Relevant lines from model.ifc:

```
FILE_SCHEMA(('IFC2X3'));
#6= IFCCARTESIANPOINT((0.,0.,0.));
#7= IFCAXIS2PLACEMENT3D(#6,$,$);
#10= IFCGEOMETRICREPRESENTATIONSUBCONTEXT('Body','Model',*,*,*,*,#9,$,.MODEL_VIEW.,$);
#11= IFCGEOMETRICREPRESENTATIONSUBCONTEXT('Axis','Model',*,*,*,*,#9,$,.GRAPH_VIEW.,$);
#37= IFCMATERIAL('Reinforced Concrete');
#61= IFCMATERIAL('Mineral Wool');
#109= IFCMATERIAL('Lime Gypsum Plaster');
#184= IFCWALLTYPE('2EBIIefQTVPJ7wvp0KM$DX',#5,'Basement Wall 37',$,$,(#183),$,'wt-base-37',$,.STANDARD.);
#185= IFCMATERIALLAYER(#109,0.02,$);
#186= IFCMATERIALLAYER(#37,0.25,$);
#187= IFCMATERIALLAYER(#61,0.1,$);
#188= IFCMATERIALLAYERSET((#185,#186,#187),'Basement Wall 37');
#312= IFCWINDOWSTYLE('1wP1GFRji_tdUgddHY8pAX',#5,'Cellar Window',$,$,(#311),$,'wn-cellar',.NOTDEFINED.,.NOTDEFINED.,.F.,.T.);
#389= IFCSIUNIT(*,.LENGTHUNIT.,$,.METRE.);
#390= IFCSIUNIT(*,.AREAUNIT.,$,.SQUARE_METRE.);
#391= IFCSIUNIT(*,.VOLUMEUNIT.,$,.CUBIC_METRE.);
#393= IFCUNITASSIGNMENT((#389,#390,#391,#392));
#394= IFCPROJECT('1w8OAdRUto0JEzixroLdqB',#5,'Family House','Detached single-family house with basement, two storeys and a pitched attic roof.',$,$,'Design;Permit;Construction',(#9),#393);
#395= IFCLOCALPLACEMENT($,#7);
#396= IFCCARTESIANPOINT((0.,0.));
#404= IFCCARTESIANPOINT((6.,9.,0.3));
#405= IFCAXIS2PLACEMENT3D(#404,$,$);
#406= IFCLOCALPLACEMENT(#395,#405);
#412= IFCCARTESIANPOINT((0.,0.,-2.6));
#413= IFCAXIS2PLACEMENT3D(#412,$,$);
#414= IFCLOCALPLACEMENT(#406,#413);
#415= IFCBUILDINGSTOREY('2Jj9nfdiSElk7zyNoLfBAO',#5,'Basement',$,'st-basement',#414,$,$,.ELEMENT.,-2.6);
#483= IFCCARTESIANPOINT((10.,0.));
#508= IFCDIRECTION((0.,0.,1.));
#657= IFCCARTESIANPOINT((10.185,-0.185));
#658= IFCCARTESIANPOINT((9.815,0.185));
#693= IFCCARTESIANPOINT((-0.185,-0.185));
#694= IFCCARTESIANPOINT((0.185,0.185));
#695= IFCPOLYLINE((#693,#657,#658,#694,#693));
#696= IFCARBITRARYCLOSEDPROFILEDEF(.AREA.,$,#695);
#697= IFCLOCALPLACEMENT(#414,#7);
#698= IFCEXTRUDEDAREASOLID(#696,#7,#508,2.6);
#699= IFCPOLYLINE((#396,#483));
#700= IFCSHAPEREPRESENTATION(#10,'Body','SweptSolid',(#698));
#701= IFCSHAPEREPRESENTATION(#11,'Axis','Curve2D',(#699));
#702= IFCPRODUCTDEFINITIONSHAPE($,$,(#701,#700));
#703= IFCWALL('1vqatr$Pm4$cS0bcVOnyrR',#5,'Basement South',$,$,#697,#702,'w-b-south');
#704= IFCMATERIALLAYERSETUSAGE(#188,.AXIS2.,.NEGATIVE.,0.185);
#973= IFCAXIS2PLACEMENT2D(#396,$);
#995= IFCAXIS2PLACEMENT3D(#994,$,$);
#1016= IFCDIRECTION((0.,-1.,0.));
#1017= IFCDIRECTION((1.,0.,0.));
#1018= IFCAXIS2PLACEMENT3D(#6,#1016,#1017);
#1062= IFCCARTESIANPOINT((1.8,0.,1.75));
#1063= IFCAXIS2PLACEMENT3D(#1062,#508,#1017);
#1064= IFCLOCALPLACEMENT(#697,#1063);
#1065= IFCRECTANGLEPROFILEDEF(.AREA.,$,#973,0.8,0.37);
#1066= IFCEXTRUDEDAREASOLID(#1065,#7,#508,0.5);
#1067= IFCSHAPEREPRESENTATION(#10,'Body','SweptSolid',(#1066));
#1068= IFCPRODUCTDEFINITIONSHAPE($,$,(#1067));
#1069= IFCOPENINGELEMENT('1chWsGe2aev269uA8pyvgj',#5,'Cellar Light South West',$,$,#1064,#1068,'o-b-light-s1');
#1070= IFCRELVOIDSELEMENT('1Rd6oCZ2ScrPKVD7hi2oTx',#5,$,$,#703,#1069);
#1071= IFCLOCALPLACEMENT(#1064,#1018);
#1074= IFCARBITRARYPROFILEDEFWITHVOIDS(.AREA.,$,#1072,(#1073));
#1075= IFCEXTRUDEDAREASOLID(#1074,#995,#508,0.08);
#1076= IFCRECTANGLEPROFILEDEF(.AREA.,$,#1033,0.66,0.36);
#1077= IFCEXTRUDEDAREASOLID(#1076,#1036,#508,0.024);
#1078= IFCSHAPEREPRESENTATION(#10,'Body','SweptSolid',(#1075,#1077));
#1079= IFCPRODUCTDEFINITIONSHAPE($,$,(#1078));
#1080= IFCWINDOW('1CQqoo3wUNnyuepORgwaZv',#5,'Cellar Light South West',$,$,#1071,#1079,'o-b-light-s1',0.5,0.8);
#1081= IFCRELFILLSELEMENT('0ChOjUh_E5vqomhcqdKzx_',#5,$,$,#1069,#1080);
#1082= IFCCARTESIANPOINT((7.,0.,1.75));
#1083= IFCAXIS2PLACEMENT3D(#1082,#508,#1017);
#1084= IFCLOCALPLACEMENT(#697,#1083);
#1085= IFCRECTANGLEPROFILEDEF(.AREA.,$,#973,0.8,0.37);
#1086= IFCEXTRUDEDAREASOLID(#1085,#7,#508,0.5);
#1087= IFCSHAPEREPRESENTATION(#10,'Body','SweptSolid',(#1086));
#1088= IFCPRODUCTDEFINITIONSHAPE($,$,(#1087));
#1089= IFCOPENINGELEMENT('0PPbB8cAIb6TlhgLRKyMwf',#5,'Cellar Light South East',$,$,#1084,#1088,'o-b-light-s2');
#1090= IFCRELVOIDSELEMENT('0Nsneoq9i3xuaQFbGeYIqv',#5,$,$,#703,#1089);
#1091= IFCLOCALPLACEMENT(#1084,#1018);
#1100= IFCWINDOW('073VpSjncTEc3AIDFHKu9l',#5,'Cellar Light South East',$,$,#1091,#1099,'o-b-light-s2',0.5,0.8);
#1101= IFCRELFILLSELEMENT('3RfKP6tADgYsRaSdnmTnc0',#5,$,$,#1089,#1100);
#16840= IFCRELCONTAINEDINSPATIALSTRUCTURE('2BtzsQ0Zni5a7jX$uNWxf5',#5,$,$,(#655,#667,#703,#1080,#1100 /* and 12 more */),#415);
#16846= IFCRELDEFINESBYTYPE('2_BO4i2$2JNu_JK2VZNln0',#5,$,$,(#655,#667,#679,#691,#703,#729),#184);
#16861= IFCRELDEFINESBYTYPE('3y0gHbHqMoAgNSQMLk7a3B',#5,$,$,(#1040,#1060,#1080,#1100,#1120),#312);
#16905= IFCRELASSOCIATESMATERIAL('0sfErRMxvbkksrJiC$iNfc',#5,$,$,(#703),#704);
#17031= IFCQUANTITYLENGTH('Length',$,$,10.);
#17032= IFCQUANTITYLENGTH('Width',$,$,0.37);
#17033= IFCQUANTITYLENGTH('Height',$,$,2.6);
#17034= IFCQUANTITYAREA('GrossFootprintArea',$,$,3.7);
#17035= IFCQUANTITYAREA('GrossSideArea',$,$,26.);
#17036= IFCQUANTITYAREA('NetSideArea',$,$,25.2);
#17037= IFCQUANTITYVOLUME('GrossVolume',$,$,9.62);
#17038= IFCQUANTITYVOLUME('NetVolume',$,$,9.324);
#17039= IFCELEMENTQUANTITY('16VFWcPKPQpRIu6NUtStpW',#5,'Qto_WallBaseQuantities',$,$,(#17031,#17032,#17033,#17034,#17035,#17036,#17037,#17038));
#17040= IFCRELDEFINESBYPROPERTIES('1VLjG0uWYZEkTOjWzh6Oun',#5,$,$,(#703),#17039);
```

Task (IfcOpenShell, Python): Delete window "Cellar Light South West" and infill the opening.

```python
import ifcopenshell
import ifcopenshell.api.feature
import ifcopenshell.api.pset
import ifcopenshell.api.root
import ifcopenshell.geom
import ifcopenshell.util.element
import ifcopenshell.util.shape
import ifcopenshell.util.unit

model = ifcopenshell.open("model.ifc")
area_scale = ifcopenshell.util.unit.calculate_unit_scale(model, "AREAUNIT")
volume_scale = ifcopenshell.util.unit.calculate_unit_scale(model, "VOLUMEUNIT")
settings = ifcopenshell.geom.settings()


def volume(element):
    """Net volume in cubic metres, openings subtracted."""
    shape = ifcopenshell.geom.create_shape(settings, element)
    return ifcopenshell.util.shape.get_volume(shape.geometry)


window = model.by_guid("1CQqoo3wUNnyuepORgwaZv")
opening = window.FillsVoids[0].RelatingOpeningElement
wall = opening.VoidsElements[0].RelatingBuildingElement
before = volume(wall)

ifcopenshell.api.root.remove_product(model, product=window)
ifcopenshell.api.feature.remove_feature(model, feature=opening)

after = volume(wall)
thickness = 0.37  # wall thickness in metres

# Update the wall's stored quantities.
qto = model.by_id(ifcopenshell.util.element.get_pset(wall, "Qto_WallBaseQuantities", should_inherit=False)["id"])
ifcopenshell.api.pset.edit_qto(model, qto=qto, properties={
    "NetSideArea": after / thickness / area_scale,
    "NetVolume": after / volume_scale,
})

print(f"wall volume {before:.3f} -> {after:.3f} m3")

model.write("model_v2.ifc")
```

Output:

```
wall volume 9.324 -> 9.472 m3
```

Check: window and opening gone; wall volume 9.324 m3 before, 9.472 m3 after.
